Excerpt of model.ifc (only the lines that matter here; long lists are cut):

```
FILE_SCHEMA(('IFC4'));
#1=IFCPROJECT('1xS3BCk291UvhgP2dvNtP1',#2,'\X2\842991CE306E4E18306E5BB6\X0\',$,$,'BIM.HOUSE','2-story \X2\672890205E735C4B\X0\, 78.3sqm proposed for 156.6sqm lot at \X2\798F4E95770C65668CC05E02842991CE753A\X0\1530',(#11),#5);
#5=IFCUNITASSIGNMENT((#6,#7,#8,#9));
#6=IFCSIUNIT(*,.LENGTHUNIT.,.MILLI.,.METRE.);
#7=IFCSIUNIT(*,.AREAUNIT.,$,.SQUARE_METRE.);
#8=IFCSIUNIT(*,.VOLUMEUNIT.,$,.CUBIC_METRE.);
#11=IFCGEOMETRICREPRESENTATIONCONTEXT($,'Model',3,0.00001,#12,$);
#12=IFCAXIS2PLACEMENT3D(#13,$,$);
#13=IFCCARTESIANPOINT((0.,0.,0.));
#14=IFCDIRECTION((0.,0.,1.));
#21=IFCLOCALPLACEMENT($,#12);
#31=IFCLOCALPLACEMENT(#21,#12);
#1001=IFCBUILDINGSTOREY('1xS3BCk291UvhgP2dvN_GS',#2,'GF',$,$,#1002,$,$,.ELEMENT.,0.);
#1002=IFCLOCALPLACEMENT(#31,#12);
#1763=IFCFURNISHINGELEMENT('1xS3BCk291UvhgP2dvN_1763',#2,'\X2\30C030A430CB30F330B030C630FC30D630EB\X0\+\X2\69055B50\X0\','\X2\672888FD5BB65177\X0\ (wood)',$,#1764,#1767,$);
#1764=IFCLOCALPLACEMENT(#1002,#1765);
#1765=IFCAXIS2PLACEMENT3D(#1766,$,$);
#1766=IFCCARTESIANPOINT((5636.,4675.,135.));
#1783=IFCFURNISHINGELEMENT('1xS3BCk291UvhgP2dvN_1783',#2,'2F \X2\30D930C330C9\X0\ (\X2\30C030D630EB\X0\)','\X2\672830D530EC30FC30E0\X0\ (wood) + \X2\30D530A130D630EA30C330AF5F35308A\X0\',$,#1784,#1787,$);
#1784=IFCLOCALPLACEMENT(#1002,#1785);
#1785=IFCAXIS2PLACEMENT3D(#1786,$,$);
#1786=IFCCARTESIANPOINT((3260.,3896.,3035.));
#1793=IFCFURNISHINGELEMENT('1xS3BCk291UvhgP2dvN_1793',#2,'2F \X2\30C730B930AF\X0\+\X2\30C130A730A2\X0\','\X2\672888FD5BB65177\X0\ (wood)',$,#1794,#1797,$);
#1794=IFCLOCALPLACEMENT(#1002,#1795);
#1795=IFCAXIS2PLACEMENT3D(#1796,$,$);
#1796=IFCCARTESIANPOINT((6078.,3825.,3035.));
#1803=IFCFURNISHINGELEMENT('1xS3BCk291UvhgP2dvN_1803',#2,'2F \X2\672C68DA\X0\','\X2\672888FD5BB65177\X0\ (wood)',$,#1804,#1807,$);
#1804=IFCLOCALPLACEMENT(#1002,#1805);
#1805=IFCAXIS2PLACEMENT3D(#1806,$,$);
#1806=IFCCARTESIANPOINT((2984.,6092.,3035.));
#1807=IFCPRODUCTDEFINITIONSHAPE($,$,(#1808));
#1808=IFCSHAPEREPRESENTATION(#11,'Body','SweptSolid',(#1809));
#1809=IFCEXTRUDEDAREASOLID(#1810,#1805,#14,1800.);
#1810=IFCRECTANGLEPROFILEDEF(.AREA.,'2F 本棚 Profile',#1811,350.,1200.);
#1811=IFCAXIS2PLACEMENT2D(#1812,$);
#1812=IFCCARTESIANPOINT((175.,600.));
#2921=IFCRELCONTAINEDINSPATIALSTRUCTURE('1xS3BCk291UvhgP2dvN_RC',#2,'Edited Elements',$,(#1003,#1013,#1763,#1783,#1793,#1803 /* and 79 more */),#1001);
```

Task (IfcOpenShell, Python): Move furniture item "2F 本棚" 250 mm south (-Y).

```python
import ifcopenshell
import ifcopenshell.api.geometry
import ifcopenshell.util.placement
import ifcopenshell.util.unit

model = ifcopenshell.open("model.ifc")
unit_scale = ifcopenshell.util.unit.calculate_unit_scale(model)

item = model.by_guid("1xS3BCk291UvhgP2dvN_1803")
matrix = ifcopenshell.util.placement.get_local_placement(item.ObjectPlacement)
matrix[1, 3] -= 0.25 / unit_scale
ifcopenshell.api.geometry.edit_object_placement(model, product=item, matrix=matrix, is_si=False)

print(ifcopenshell.util.placement.get_local_placement(item.ObjectPlacement).round(3) + 0.0)

model.write("model-out.ifc")
```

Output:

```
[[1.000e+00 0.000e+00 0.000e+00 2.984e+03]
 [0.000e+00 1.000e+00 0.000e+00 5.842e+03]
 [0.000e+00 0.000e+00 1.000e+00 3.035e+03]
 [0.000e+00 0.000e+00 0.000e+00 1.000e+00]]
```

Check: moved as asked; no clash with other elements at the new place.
